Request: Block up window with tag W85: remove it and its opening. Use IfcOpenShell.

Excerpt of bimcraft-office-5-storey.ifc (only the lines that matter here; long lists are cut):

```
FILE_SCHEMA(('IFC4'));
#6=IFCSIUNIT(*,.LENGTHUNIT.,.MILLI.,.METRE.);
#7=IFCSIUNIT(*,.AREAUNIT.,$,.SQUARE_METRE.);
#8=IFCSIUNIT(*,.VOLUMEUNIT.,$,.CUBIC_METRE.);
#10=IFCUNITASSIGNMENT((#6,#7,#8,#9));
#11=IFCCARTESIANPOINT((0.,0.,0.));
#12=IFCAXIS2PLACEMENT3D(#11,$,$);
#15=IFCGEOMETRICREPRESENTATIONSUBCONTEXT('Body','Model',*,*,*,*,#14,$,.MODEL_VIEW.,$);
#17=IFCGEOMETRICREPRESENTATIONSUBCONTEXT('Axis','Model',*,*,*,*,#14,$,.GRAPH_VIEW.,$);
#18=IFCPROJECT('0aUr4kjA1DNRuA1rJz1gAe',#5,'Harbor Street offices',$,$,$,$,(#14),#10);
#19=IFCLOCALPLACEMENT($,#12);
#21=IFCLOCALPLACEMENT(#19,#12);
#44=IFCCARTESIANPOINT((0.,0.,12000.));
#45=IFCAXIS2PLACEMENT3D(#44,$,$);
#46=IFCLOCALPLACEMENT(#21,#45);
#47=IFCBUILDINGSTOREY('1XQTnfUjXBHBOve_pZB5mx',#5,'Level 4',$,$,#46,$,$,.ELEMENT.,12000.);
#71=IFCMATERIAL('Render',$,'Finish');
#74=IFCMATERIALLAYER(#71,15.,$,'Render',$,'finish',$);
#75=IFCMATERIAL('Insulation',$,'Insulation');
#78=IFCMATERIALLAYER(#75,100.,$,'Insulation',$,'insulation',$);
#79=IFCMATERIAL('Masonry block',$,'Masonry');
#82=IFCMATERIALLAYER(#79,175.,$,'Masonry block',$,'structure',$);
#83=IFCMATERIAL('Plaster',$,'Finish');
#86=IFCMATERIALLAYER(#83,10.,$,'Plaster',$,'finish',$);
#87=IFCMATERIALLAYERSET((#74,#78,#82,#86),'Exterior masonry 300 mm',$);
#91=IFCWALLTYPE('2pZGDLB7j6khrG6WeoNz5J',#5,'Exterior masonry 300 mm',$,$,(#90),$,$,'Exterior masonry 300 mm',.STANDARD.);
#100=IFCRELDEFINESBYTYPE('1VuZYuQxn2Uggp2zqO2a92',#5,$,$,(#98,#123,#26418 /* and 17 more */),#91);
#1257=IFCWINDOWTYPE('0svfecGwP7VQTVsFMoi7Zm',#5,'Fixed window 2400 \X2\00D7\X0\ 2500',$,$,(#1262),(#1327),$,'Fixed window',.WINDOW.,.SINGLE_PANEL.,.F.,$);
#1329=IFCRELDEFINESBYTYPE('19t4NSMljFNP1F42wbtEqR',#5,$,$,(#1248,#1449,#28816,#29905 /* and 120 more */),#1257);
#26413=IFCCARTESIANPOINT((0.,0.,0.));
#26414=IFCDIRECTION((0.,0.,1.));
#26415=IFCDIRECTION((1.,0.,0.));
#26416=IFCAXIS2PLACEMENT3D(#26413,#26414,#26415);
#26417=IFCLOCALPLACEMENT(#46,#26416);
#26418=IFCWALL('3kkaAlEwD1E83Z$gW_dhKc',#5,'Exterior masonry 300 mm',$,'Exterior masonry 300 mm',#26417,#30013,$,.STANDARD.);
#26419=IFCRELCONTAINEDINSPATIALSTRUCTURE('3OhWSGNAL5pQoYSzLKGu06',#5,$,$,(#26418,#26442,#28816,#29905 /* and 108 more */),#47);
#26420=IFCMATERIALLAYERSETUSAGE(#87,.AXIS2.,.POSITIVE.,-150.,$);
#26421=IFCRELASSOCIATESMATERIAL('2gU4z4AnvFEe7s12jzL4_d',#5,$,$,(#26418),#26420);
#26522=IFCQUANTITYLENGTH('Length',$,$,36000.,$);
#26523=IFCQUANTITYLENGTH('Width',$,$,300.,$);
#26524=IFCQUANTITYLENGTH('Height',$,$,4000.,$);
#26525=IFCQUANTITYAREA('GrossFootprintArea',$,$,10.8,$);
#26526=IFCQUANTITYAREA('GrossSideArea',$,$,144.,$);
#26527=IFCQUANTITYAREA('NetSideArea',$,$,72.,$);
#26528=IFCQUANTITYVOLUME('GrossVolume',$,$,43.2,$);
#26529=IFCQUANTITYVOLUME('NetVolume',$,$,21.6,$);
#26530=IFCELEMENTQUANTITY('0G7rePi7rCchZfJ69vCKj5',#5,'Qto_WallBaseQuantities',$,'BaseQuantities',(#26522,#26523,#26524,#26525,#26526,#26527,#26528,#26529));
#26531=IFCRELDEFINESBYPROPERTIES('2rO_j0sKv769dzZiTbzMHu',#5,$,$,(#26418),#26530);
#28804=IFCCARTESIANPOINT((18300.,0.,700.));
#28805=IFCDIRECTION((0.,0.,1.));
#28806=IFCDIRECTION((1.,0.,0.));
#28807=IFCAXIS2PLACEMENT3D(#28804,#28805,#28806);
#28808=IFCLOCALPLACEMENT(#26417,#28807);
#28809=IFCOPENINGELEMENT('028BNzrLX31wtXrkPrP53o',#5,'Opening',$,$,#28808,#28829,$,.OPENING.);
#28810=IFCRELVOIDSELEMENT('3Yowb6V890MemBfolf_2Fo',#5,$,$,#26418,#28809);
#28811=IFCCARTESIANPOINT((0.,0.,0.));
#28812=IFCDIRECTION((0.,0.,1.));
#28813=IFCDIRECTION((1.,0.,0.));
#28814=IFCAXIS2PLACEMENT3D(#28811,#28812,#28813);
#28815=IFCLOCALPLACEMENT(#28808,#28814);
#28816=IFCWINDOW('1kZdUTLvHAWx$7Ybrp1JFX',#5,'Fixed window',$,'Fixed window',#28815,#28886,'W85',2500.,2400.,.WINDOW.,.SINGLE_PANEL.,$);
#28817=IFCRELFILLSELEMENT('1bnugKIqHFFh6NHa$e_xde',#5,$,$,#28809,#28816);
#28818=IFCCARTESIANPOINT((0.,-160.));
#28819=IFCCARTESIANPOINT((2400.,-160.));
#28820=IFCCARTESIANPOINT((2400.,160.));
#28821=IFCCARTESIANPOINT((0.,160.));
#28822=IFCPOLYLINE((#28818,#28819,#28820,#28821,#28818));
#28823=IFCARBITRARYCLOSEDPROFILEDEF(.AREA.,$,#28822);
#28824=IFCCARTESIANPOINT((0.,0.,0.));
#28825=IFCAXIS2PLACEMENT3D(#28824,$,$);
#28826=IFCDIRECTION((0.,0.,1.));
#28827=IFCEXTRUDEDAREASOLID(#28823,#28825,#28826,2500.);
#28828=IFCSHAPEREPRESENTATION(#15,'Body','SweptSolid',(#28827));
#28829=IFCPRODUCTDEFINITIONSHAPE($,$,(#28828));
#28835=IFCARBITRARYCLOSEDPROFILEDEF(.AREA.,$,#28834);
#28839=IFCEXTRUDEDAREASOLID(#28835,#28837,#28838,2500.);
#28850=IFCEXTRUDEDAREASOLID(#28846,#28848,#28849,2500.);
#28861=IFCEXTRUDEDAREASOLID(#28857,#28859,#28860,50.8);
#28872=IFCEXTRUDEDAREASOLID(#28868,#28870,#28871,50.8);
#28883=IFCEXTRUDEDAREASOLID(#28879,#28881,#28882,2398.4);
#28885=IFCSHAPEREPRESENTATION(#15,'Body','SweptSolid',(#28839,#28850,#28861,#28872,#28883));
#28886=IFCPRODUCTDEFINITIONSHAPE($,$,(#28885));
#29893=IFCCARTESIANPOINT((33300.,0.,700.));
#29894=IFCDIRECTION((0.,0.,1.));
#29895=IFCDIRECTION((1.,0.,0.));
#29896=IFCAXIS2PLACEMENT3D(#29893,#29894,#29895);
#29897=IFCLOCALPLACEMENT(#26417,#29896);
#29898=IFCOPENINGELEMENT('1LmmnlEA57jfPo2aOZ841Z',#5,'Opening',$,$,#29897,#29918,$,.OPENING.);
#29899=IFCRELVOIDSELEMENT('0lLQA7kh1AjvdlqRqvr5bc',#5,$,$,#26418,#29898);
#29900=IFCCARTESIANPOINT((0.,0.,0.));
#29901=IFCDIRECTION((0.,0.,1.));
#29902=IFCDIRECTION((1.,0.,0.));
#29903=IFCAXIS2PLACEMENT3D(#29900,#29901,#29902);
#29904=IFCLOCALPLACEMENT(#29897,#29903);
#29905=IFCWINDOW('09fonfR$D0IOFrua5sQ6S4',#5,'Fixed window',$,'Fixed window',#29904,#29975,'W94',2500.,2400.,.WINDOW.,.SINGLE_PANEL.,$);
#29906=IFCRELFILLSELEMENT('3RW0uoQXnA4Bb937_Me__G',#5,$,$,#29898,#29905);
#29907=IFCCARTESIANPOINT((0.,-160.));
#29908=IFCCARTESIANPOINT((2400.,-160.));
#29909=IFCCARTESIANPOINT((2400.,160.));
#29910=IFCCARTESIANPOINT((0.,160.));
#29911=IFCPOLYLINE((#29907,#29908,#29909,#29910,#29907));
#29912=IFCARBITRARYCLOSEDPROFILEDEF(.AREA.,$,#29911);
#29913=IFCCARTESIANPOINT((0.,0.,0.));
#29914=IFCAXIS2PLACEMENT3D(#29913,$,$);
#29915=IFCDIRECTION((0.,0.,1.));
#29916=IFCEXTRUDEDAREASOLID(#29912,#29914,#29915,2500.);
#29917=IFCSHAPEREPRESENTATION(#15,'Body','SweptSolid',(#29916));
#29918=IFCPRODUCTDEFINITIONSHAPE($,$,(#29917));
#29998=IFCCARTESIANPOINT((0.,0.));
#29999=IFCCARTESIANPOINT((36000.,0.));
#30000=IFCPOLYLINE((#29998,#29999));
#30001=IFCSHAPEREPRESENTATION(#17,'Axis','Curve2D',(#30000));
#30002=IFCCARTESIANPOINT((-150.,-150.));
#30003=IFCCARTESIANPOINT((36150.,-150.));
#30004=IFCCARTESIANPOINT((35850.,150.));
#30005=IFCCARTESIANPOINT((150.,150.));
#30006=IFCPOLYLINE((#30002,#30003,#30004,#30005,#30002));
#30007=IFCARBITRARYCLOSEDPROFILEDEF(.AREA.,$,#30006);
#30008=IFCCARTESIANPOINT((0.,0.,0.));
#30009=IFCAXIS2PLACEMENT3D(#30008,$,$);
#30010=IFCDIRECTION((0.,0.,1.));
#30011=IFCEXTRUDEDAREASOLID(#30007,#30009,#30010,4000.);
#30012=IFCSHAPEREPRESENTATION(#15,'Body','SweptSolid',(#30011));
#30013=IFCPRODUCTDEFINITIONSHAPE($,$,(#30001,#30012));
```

```python
import ifcopenshell
import ifcopenshell.api.feature
import ifcopenshell.api.pset
import ifcopenshell.api.root
import ifcopenshell.geom
import ifcopenshell.util.element
import ifcopenshell.util.shape
import ifcopenshell.util.unit

model = ifcopenshell.open("bimcraft-office-5-storey.ifc")
area_scale = ifcopenshell.util.unit.calculate_unit_scale(model, "AREAUNIT")
volume_scale = ifcopenshell.util.unit.calculate_unit_scale(model, "VOLUMEUNIT")
settings = ifcopenshell.geom.settings()


def volume(element):
    """Net volume in cubic metres, openings subtracted."""
    shape = ifcopenshell.geom.create_shape(settings, element)
    return ifcopenshell.util.shape.get_volume(shape.geometry)


window = model.by_guid("1kZdUTLvHAWx$7Ybrp1JFX")
opening = window.FillsVoids[0].RelatingOpeningElement
wall = opening.VoidsElements[0].RelatingBuildingElement
before = volume(wall)

ifcopenshell.api.root.remove_product(model, product=window)
ifcopenshell.api.feature.remove_feature(model, feature=opening)

after = volume(wall)
thickness = 0.3  # wall thickness in metres

# Update the wall's stored quantities.
qto = model.by_id(ifcopenshell.util.element.get_pset(wall, "Qto_WallBaseQuantities", should_inherit=False)["id"])
ifcopenshell.api.pset.edit_qto(model, qto=qto, properties={
    "NetSideArea": after / thickness / area_scale,
    "NetVolume": after / volume_scale,
})

print(f"wall volume {before:.3f} -> {after:.3f} m3")

model.write("bimcraft-office-5-storey-out.ifc")
```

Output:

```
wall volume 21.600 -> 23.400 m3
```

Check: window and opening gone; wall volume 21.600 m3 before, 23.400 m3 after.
